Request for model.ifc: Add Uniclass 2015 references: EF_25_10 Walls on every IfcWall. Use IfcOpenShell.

First a look at what the model holds.

```python
import ifcopenshell

model = ifcopenshell.open("model.ifc")
print(model.schema)
print("classifications:", [c.Name for c in model.by_type("IfcClassification")])
for ifc_class in ("IfcDoor", "IfcRoof", "IfcStair", "IfcWall", "IfcWindow"):
    print(ifc_class, len(model.by_type(ifc_class)))
```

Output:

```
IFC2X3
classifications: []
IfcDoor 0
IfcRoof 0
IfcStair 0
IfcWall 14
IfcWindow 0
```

```python
import ifcopenshell
import ifcopenshell.api.classification

model = ifcopenshell.open("model.ifc")

# IFC2X3 requires Source and Edition and has no link from the project to the system.
system = model.create_entity("IfcClassification", Source="NBS", Edition="2015", Name="Uniclass 2015")

codes = {
    "IfcWall": ("EF_25_10", "Walls"),
}
for ifc_class, (code, name) in codes.items():
    products = model.by_type(ifc_class)
    ifcopenshell.api.classification.add_reference(
        model, products=products, classification=system, identification=code, name=name
    )
    print(code, len(products))

model.write("model-out.ifc")
```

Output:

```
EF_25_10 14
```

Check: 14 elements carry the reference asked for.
